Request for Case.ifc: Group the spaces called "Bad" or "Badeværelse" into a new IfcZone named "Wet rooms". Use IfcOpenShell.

First a look at what the model holds.

```python
import ifcopenshell

model = ifcopenshell.open("Case.ifc")
print(model.schema)
seen = {}
for space in model.by_type("IfcSpace"):
    seen[space.LongName] = seen.get(space.LongName, 0) + 1
for name, count in sorted(seen.items(), key=str):
    print(count, "x", name)
print("zones:", [z.Name for z in model.by_type("IfcZone")][:20])
```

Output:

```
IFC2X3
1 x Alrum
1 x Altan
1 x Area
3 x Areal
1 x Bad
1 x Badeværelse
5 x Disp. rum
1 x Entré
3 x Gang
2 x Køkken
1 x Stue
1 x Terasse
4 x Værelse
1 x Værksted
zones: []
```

```python
import ifcopenshell
import ifcopenshell.api.group
import ifcopenshell.api.root

model = ifcopenshell.open("Case.ifc")

names = {"Bad", "Badeværelse"}
spaces = [s for s in model.by_type("IfcSpace") if s.LongName in names]

zone = ifcopenshell.api.root.create_entity(model, ifc_class="IfcZone", name="Wet rooms")
ifcopenshell.api.group.assign_group(model, products=spaces, group=zone)
print(len(spaces), "spaces in", zone.Name)

model.write("Case_edited.ifc")
```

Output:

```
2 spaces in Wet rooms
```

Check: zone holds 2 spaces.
